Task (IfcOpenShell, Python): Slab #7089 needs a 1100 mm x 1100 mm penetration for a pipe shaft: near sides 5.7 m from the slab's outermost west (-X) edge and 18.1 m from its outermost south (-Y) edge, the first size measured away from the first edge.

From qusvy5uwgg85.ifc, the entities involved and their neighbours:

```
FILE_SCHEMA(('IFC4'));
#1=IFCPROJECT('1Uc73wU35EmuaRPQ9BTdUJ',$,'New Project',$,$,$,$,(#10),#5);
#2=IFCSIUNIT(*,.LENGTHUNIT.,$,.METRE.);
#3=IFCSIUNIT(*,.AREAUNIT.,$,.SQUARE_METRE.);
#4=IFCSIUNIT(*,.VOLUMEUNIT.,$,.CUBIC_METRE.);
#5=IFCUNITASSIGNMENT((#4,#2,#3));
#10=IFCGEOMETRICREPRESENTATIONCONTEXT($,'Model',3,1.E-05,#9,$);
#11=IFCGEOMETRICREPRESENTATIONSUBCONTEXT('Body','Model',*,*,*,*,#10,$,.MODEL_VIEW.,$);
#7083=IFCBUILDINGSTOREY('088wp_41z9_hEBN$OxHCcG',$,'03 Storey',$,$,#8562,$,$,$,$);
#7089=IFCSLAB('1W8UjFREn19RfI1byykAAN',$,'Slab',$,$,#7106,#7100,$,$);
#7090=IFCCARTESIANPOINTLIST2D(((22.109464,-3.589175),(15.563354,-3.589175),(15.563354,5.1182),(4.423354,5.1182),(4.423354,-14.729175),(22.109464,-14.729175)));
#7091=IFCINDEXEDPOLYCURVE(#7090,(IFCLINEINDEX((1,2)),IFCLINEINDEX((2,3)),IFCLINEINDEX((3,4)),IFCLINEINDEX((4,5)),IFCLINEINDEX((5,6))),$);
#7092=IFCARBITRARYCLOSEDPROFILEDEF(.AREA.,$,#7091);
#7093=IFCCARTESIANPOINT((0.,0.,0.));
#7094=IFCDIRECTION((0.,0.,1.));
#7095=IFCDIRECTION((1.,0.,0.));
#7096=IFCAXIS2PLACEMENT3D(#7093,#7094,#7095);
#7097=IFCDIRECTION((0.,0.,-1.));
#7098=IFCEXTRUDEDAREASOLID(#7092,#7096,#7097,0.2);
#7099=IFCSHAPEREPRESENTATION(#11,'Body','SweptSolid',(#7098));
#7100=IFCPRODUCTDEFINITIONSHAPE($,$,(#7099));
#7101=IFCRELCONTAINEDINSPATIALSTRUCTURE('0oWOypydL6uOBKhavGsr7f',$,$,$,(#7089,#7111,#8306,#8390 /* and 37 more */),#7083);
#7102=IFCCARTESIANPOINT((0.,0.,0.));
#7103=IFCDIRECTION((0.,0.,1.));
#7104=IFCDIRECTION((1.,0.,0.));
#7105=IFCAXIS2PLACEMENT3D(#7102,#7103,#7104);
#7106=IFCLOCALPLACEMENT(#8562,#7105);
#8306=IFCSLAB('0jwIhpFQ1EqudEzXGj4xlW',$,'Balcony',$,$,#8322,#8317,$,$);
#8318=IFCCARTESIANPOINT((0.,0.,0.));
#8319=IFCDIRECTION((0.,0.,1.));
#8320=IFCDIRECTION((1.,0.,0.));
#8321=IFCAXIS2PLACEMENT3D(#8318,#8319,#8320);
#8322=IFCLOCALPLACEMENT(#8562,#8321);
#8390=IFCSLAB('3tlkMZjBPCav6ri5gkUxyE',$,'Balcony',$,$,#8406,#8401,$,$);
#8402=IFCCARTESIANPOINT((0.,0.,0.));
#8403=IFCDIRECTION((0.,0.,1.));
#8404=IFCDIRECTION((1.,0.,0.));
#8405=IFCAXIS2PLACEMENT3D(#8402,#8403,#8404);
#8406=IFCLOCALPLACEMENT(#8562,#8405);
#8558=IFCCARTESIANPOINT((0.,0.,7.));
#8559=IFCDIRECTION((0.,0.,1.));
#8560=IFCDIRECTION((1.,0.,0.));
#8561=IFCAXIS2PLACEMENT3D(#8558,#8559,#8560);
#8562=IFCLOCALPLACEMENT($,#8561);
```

```python
import numpy as np
import ifcopenshell
import ifcopenshell.api.feature
import ifcopenshell.api.geometry
import ifcopenshell.api.root
import ifcopenshell.geom
import ifcopenshell.util.placement
import ifcopenshell.util.representation
import ifcopenshell.util.shape
import ifcopenshell.util.unit

model = ifcopenshell.open("qusvy5uwgg85.ifc")
unit_scale = ifcopenshell.util.unit.calculate_unit_scale(model)
settings = ifcopenshell.geom.settings()


def volume(element):
    """Net volume in cubic metres, openings subtracted."""
    shape = ifcopenshell.geom.create_shape(settings, element)
    return ifcopenshell.util.shape.get_volume(shape.geometry)


slab = model.by_guid("1W8UjFREn19RfI1byykAAN")
before = volume(slab)

# Extent in the slab's own axes, in metres. The edges named are its -X and -Y sides.
slab_shape = ifcopenshell.geom.create_shape(settings, slab)
vertices = ifcopenshell.util.shape.get_vertices(slab_shape.geometry)
x_min, y_min, bottom = vertices.min(axis=0)
top = vertices[:, 2].max()

opening = ifcopenshell.api.root.create_entity(model, ifc_class="IfcOpeningElement", name="Pipe shaft opening", predefined_type="OPENING")
context = ifcopenshell.util.representation.get_context(model, "Model", "Body", "MODEL_VIEW")
width, depth = 1.1, 1.1
outline = [(0.0, 0.0), (width, 0.0), (width, depth), (0.0, depth), (0.0, 0.0)]
# Overshoot both faces by 50 mm so the cut is clean.
shape = ifcopenshell.api.geometry.add_slab_representation(
    model, context=context, depth=top - bottom + 0.1, polyline=outline
)
ifcopenshell.api.geometry.assign_representation(model, product=opening, representation=shape)

matrix = ifcopenshell.util.placement.get_local_placement(slab.ObjectPlacement)
matrix[:, 3] = matrix @ np.append(np.array([x_min + 5.7, y_min + 18.1, bottom - 0.05]) / unit_scale, 1.0)
ifcopenshell.api.geometry.edit_object_placement(model, product=opening, matrix=matrix, is_si=False)
ifcopenshell.api.feature.add_feature(model, feature=opening, element=slab)

after = volume(slab)

print(f"slab volume {before:.3f} -> {after:.3f} m3")

model.write("qusvy5uwgg85_edited.ifc")
```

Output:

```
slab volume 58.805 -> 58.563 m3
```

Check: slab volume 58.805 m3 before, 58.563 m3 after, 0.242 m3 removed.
